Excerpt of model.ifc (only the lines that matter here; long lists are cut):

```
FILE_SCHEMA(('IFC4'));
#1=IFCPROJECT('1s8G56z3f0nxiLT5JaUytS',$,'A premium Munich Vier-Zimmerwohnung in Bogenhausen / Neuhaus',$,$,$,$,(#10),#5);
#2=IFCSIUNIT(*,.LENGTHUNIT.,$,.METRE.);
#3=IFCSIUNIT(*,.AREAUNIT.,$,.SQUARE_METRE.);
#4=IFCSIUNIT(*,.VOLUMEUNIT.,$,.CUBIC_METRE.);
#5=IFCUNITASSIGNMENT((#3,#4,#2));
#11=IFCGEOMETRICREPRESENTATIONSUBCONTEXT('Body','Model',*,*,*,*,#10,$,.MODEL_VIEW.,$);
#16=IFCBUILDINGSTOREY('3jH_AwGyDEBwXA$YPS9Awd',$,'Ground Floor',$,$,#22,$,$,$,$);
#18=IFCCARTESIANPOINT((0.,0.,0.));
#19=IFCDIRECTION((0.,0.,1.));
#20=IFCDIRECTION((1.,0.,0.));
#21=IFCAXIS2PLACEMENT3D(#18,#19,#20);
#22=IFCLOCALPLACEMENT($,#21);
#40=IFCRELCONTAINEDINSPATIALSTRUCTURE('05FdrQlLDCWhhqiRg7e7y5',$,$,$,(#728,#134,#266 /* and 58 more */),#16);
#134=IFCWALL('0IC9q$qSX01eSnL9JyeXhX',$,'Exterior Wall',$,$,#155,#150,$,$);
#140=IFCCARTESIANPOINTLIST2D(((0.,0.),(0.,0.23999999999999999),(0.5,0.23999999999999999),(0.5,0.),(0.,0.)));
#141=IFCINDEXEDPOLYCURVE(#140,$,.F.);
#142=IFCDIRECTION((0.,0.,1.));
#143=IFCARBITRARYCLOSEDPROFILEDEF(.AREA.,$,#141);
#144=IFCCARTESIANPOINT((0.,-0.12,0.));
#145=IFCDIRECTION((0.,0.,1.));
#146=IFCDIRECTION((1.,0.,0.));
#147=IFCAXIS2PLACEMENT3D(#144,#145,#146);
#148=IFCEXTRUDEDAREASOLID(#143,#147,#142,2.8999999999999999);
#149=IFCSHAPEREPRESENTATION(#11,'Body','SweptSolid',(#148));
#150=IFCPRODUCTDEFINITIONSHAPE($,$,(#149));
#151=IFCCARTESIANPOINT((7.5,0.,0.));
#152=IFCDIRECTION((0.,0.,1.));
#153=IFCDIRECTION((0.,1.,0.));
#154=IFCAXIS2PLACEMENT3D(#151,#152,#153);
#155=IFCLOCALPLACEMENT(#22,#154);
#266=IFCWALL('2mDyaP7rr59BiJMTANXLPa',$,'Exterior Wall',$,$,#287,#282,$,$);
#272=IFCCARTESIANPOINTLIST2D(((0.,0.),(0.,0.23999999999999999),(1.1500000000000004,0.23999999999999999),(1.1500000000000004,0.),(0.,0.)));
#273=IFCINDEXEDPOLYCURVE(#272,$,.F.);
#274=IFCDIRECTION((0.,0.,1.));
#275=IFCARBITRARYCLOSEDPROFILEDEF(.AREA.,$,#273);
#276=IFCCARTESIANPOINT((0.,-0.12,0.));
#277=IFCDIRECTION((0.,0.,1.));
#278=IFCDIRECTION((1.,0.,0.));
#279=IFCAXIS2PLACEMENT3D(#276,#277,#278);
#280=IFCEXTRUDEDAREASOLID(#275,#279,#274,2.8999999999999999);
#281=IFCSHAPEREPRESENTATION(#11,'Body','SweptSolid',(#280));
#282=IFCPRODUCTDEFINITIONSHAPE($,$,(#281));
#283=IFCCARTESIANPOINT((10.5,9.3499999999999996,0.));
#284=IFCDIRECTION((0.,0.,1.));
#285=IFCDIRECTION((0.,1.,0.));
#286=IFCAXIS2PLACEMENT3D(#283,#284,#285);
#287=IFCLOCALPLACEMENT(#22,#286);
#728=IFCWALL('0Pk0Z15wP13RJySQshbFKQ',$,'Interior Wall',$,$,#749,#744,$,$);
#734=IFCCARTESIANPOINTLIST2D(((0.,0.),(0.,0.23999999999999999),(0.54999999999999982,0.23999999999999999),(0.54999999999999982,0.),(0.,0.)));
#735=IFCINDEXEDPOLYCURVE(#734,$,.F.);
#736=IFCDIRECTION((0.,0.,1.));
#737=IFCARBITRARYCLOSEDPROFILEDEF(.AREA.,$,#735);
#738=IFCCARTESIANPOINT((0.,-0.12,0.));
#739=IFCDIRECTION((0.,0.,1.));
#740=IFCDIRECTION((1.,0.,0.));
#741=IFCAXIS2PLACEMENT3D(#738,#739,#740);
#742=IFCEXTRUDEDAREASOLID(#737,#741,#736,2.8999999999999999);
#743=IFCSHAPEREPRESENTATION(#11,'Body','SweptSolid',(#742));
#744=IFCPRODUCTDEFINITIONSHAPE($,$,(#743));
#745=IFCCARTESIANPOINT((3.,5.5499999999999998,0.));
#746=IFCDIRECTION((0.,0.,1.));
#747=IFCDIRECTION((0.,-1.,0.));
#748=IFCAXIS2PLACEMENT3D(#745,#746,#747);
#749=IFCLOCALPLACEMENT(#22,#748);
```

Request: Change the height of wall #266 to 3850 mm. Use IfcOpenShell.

```python
import ifcopenshell
import ifcopenshell.geom
import ifcopenshell.util.representation
import ifcopenshell.util.shape

model = ifcopenshell.open("model.ifc")
settings = ifcopenshell.geom.settings()


def volume(element):
    """Net volume in cubic metres, openings subtracted."""
    shape = ifcopenshell.geom.create_shape(settings, element)
    return ifcopenshell.util.shape.get_volume(shape.geometry)


wall = model.by_guid("2mDyaP7rr59BiJMTANXLPa")
before = volume(wall)

body = ifcopenshell.util.representation.get_representation(wall, "Model", "Body")
solid = body.Items[0]
old_height = solid.Depth
solid.Depth = 3.85
after = volume(wall)

print(f"height {old_height:g} -> {solid.Depth:g}, volume {before:.3f} -> {after:.3f} m3")

model.write("model_updated.ifc")
```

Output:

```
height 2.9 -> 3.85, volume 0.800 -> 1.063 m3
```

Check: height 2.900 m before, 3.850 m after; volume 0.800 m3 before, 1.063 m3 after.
